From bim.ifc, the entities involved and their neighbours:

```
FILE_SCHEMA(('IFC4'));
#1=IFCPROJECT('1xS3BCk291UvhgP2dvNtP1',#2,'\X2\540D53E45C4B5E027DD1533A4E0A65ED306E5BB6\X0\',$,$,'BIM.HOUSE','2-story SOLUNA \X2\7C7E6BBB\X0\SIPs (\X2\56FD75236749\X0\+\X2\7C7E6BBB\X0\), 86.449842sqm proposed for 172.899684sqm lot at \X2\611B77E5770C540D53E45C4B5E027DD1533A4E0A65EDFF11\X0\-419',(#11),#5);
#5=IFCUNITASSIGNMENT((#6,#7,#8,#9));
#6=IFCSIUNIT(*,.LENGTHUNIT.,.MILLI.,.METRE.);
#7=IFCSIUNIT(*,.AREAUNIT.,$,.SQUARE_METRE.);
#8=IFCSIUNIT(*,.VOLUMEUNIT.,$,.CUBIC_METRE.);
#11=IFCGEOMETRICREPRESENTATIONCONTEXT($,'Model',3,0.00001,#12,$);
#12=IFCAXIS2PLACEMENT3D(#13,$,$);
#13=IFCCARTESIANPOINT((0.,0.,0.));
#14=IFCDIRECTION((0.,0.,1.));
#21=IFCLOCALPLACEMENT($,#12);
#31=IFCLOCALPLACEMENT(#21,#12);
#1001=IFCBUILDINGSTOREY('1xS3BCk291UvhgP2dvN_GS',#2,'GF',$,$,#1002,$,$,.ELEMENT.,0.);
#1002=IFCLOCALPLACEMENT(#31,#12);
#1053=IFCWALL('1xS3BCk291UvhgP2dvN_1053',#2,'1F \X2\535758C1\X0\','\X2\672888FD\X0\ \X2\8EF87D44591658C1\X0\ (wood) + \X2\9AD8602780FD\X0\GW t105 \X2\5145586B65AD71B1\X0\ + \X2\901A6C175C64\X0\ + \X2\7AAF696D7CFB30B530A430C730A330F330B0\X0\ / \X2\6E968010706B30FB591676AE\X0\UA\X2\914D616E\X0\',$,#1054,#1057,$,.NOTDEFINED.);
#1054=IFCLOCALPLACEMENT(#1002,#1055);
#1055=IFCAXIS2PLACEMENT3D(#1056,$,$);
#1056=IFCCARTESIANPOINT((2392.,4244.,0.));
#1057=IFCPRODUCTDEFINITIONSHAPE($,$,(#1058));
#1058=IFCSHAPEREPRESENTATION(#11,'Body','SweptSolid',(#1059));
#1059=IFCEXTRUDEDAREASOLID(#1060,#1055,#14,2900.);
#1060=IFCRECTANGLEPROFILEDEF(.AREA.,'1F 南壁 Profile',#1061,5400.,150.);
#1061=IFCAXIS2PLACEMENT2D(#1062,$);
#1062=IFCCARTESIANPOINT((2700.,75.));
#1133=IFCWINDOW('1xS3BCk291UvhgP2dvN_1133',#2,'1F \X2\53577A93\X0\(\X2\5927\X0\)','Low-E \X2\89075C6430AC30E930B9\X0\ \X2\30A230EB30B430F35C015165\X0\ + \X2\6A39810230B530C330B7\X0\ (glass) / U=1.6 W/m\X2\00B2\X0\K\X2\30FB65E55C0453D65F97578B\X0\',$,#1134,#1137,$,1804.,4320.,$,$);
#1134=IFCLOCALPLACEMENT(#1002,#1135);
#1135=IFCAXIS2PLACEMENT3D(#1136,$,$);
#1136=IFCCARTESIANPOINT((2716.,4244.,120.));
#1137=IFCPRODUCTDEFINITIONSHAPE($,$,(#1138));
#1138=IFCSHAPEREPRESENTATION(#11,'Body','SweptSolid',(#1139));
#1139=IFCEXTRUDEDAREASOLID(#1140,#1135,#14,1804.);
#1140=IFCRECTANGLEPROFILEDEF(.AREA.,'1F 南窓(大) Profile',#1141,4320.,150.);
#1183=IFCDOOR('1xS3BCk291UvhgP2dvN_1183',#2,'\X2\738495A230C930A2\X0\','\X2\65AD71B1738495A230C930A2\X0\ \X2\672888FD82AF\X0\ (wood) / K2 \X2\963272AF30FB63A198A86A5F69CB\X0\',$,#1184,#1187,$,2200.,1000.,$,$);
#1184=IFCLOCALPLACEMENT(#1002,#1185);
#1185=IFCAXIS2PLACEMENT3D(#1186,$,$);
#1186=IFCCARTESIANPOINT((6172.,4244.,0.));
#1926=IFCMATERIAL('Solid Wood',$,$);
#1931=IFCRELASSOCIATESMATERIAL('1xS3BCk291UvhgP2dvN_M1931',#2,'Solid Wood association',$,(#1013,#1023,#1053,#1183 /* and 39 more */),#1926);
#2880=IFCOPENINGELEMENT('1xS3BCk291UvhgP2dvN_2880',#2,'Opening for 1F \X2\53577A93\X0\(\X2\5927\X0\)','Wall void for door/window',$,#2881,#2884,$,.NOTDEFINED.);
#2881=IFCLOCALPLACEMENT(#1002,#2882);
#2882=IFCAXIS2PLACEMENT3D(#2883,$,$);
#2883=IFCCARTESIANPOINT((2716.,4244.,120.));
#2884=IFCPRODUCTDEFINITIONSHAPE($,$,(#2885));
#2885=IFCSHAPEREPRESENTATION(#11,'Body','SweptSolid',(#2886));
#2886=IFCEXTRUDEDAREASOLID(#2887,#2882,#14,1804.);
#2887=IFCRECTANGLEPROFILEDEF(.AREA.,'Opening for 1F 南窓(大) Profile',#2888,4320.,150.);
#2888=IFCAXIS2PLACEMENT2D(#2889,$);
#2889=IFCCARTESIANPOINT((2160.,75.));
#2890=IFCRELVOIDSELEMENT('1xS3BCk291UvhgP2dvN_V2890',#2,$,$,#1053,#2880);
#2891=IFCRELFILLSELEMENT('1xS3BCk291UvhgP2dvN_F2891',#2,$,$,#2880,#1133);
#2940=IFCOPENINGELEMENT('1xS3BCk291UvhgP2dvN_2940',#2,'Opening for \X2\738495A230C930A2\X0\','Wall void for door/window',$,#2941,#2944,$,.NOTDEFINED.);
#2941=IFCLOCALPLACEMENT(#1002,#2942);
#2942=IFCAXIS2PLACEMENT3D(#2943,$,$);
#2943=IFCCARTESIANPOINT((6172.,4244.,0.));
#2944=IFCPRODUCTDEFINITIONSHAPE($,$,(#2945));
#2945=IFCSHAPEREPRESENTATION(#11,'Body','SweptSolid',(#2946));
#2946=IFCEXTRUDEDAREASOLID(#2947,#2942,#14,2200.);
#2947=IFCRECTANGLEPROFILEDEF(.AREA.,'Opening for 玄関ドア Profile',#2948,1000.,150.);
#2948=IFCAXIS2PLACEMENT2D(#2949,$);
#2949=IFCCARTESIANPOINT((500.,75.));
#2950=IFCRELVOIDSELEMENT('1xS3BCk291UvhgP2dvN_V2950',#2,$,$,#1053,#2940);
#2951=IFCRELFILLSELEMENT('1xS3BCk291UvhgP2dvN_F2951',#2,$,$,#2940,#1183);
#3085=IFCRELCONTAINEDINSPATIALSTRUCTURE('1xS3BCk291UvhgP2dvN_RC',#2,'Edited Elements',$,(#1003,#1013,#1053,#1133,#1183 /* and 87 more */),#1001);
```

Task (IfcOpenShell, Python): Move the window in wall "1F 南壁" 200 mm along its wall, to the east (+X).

```python
import ifcopenshell
import ifcopenshell.api.geometry
import ifcopenshell.util.placement

model = ifcopenshell.open("bim.ifc")

window = model.by_guid("1xS3BCk291UvhgP2dvN_1133")
opening = window.FillsVoids[0].RelatingOpeningElement
wall = opening.VoidsElements[0].RelatingBuildingElement

wall_matrix = ifcopenshell.util.placement.get_local_placement(wall.ObjectPlacement)
shift = wall_matrix[:3, 0] * 200.0
before = ifcopenshell.util.placement.get_local_placement(window.ObjectPlacement)[:3, 3].copy()

# The window is not placed relative to its opening, so move both.
for product in (opening, window):
    matrix = ifcopenshell.util.placement.get_local_placement(product.ObjectPlacement)
    matrix[:3, 3] += shift
    ifcopenshell.api.geometry.edit_object_placement(model, product=product, matrix=matrix, is_si=False)

after = ifcopenshell.util.placement.get_local_placement(window.ObjectPlacement)[:3, 3]
print("window moved by", (after - before).round(3) + 0.0)

model.write("bim_updated.ifc")
```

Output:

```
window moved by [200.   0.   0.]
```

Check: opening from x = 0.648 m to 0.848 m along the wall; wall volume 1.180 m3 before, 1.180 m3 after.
